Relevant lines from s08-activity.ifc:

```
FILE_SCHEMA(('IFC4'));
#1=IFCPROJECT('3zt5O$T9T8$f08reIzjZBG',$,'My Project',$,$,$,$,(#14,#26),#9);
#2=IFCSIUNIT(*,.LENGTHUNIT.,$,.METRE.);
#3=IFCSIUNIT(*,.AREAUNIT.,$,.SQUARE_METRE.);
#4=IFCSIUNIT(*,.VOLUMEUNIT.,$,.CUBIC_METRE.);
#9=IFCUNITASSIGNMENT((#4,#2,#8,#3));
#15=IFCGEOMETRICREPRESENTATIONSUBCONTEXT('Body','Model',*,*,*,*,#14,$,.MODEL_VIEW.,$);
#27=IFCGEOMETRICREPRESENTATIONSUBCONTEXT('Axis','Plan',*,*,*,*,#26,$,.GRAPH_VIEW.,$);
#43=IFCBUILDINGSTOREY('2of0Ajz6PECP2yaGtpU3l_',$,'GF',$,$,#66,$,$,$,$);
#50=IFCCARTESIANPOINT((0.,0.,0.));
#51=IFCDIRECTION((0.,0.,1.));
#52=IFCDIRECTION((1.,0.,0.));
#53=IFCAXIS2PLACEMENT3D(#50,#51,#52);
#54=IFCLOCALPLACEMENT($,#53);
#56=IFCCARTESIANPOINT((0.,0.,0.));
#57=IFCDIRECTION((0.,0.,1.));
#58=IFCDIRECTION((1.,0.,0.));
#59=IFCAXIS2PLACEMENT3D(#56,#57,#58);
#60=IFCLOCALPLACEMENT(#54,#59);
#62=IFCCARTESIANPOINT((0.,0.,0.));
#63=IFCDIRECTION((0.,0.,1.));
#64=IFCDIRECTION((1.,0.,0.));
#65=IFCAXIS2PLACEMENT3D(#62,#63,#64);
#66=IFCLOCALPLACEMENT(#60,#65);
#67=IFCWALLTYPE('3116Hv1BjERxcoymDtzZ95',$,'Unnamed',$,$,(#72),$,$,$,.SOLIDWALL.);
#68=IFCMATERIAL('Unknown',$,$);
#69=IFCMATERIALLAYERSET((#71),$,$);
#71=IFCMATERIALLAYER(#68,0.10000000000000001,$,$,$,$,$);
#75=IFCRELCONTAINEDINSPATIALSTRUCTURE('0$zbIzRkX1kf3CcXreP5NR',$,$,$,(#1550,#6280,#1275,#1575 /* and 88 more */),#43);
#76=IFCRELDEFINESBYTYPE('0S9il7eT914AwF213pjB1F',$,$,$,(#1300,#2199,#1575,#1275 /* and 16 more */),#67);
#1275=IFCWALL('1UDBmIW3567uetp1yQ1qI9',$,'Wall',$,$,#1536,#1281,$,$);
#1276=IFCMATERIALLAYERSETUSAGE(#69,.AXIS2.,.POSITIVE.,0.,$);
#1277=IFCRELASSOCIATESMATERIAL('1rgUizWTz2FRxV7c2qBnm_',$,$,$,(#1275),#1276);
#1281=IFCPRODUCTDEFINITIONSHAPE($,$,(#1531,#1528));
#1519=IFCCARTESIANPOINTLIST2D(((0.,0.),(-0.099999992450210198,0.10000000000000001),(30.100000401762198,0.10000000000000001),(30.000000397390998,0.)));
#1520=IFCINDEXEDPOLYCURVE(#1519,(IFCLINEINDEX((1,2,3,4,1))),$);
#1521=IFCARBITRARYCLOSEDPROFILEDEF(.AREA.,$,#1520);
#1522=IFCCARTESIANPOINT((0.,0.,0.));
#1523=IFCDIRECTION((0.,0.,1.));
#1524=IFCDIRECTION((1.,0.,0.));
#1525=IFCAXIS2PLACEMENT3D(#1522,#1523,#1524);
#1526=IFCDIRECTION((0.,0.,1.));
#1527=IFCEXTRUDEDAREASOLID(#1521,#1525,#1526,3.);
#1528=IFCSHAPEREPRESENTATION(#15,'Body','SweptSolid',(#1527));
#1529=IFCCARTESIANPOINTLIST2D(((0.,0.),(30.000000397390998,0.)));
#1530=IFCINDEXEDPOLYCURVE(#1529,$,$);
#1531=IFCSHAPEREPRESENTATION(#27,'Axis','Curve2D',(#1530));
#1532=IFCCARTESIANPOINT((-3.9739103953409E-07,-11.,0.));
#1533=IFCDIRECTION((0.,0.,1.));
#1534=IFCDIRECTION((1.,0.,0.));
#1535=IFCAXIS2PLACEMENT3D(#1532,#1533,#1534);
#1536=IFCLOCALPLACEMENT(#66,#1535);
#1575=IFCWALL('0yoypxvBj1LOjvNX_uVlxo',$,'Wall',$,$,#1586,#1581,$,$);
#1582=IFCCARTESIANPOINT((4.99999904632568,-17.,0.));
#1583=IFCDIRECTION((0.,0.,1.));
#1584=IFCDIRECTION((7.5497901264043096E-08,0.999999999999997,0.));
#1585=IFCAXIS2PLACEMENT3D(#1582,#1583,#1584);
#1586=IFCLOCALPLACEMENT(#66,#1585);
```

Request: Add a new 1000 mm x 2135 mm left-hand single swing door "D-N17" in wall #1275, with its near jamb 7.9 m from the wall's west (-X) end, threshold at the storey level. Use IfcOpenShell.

```python
import numpy as np
import ifcopenshell
import ifcopenshell.api.feature
import ifcopenshell.api.geometry
import ifcopenshell.api.root
import ifcopenshell.api.spatial
import ifcopenshell.geom
import ifcopenshell.util.element
import ifcopenshell.util.placement
import ifcopenshell.util.representation
import ifcopenshell.util.shape
import ifcopenshell.util.unit

model = ifcopenshell.open("s08-activity.ifc")
unit_scale = ifcopenshell.util.unit.calculate_unit_scale(model)
settings = ifcopenshell.geom.settings()


def volume(element):
    """Net volume in cubic metres, openings subtracted."""
    shape = ifcopenshell.geom.create_shape(settings, element)
    return ifcopenshell.util.shape.get_volume(shape.geometry)


wall = model.by_guid("1UDBmIW3567uetp1yQ1qI9")
storey = ifcopenshell.util.element.get_container(wall, ifc_class="IfcBuildingStorey")
context = ifcopenshell.util.representation.get_context(model, "Model", "Body", "MODEL_VIEW")
before = volume(wall)

width, height, from_end, sill = 1, 2.135, 7.9, 0.0  # metres

# The wall runs along its own X axis, and the end named is its -X end.
wall_shape = ifcopenshell.geom.create_shape(settings, wall)
x, y, z = ifcopenshell.util.shape.get_vertices(wall_shape.geometry).T
start = x.min() + from_end
face, thickness = float(y.min()), float(y.max() - y.min())
wall_matrix = ifcopenshell.util.placement.get_local_placement(wall.ObjectPlacement)
level = ifcopenshell.util.placement.get_local_placement(storey.ObjectPlacement)[2, 3]


def in_wall(x, y):
    """Placement at x, y metres in the wall's axes, at sill height."""
    matrix = wall_matrix.copy()
    matrix[:, 3] = wall_matrix @ np.array([x / unit_scale, y / unit_scale, 0.0, 1.0])
    matrix[2, 3] = level + sill / unit_scale
    return matrix


# Opening: a box that overshoots both wall faces by 50 mm.
opening = ifcopenshell.api.root.create_entity(model, ifc_class="IfcOpeningElement", predefined_type="OPENING")
box = ifcopenshell.api.geometry.add_wall_representation(
    model, context=context, length=width, height=height, thickness=thickness + 0.1
)
ifcopenshell.api.geometry.assign_representation(model, product=opening, representation=box)
ifcopenshell.api.geometry.edit_object_placement(model, product=opening, matrix=in_wall(start, face - 0.05), is_si=False)
ifcopenshell.api.feature.add_feature(model, feature=opening, element=wall)

door = ifcopenshell.api.root.create_entity(model, ifc_class="IfcDoor", name="D-N17", predefined_type="DOOR")
door.OverallWidth, door.OverallHeight = width / unit_scale, height / unit_scale
door.OperationType = "SINGLE_SWING_LEFT"
body = ifcopenshell.api.geometry.add_door_representation(
    model,
    context=context,
    overall_width=door.OverallWidth,
    overall_height=door.OverallHeight,
    operation_type="SINGLE_SWING_LEFT",
    lining_properties={"LiningDepth": thickness / unit_scale, "ThresholdDepth": thickness / unit_scale},
)
ifcopenshell.api.geometry.assign_representation(model, product=door, representation=body)
ifcopenshell.api.spatial.assign_container(model, products=[door], relating_structure=storey)
ifcopenshell.api.feature.add_filling(model, opening=opening, element=door)

# The lining spans the wall, so the door starts at the wall face.
ifcopenshell.api.geometry.edit_object_placement(model, product=door, matrix=in_wall(start, face), is_si=False)

after = volume(wall)

print(f"wall volume {before:.3f} -> {after:.3f} m3")

model.write("s08-activity_rev.ifc")
```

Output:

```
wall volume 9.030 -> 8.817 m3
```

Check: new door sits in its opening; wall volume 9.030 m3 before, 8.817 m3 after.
